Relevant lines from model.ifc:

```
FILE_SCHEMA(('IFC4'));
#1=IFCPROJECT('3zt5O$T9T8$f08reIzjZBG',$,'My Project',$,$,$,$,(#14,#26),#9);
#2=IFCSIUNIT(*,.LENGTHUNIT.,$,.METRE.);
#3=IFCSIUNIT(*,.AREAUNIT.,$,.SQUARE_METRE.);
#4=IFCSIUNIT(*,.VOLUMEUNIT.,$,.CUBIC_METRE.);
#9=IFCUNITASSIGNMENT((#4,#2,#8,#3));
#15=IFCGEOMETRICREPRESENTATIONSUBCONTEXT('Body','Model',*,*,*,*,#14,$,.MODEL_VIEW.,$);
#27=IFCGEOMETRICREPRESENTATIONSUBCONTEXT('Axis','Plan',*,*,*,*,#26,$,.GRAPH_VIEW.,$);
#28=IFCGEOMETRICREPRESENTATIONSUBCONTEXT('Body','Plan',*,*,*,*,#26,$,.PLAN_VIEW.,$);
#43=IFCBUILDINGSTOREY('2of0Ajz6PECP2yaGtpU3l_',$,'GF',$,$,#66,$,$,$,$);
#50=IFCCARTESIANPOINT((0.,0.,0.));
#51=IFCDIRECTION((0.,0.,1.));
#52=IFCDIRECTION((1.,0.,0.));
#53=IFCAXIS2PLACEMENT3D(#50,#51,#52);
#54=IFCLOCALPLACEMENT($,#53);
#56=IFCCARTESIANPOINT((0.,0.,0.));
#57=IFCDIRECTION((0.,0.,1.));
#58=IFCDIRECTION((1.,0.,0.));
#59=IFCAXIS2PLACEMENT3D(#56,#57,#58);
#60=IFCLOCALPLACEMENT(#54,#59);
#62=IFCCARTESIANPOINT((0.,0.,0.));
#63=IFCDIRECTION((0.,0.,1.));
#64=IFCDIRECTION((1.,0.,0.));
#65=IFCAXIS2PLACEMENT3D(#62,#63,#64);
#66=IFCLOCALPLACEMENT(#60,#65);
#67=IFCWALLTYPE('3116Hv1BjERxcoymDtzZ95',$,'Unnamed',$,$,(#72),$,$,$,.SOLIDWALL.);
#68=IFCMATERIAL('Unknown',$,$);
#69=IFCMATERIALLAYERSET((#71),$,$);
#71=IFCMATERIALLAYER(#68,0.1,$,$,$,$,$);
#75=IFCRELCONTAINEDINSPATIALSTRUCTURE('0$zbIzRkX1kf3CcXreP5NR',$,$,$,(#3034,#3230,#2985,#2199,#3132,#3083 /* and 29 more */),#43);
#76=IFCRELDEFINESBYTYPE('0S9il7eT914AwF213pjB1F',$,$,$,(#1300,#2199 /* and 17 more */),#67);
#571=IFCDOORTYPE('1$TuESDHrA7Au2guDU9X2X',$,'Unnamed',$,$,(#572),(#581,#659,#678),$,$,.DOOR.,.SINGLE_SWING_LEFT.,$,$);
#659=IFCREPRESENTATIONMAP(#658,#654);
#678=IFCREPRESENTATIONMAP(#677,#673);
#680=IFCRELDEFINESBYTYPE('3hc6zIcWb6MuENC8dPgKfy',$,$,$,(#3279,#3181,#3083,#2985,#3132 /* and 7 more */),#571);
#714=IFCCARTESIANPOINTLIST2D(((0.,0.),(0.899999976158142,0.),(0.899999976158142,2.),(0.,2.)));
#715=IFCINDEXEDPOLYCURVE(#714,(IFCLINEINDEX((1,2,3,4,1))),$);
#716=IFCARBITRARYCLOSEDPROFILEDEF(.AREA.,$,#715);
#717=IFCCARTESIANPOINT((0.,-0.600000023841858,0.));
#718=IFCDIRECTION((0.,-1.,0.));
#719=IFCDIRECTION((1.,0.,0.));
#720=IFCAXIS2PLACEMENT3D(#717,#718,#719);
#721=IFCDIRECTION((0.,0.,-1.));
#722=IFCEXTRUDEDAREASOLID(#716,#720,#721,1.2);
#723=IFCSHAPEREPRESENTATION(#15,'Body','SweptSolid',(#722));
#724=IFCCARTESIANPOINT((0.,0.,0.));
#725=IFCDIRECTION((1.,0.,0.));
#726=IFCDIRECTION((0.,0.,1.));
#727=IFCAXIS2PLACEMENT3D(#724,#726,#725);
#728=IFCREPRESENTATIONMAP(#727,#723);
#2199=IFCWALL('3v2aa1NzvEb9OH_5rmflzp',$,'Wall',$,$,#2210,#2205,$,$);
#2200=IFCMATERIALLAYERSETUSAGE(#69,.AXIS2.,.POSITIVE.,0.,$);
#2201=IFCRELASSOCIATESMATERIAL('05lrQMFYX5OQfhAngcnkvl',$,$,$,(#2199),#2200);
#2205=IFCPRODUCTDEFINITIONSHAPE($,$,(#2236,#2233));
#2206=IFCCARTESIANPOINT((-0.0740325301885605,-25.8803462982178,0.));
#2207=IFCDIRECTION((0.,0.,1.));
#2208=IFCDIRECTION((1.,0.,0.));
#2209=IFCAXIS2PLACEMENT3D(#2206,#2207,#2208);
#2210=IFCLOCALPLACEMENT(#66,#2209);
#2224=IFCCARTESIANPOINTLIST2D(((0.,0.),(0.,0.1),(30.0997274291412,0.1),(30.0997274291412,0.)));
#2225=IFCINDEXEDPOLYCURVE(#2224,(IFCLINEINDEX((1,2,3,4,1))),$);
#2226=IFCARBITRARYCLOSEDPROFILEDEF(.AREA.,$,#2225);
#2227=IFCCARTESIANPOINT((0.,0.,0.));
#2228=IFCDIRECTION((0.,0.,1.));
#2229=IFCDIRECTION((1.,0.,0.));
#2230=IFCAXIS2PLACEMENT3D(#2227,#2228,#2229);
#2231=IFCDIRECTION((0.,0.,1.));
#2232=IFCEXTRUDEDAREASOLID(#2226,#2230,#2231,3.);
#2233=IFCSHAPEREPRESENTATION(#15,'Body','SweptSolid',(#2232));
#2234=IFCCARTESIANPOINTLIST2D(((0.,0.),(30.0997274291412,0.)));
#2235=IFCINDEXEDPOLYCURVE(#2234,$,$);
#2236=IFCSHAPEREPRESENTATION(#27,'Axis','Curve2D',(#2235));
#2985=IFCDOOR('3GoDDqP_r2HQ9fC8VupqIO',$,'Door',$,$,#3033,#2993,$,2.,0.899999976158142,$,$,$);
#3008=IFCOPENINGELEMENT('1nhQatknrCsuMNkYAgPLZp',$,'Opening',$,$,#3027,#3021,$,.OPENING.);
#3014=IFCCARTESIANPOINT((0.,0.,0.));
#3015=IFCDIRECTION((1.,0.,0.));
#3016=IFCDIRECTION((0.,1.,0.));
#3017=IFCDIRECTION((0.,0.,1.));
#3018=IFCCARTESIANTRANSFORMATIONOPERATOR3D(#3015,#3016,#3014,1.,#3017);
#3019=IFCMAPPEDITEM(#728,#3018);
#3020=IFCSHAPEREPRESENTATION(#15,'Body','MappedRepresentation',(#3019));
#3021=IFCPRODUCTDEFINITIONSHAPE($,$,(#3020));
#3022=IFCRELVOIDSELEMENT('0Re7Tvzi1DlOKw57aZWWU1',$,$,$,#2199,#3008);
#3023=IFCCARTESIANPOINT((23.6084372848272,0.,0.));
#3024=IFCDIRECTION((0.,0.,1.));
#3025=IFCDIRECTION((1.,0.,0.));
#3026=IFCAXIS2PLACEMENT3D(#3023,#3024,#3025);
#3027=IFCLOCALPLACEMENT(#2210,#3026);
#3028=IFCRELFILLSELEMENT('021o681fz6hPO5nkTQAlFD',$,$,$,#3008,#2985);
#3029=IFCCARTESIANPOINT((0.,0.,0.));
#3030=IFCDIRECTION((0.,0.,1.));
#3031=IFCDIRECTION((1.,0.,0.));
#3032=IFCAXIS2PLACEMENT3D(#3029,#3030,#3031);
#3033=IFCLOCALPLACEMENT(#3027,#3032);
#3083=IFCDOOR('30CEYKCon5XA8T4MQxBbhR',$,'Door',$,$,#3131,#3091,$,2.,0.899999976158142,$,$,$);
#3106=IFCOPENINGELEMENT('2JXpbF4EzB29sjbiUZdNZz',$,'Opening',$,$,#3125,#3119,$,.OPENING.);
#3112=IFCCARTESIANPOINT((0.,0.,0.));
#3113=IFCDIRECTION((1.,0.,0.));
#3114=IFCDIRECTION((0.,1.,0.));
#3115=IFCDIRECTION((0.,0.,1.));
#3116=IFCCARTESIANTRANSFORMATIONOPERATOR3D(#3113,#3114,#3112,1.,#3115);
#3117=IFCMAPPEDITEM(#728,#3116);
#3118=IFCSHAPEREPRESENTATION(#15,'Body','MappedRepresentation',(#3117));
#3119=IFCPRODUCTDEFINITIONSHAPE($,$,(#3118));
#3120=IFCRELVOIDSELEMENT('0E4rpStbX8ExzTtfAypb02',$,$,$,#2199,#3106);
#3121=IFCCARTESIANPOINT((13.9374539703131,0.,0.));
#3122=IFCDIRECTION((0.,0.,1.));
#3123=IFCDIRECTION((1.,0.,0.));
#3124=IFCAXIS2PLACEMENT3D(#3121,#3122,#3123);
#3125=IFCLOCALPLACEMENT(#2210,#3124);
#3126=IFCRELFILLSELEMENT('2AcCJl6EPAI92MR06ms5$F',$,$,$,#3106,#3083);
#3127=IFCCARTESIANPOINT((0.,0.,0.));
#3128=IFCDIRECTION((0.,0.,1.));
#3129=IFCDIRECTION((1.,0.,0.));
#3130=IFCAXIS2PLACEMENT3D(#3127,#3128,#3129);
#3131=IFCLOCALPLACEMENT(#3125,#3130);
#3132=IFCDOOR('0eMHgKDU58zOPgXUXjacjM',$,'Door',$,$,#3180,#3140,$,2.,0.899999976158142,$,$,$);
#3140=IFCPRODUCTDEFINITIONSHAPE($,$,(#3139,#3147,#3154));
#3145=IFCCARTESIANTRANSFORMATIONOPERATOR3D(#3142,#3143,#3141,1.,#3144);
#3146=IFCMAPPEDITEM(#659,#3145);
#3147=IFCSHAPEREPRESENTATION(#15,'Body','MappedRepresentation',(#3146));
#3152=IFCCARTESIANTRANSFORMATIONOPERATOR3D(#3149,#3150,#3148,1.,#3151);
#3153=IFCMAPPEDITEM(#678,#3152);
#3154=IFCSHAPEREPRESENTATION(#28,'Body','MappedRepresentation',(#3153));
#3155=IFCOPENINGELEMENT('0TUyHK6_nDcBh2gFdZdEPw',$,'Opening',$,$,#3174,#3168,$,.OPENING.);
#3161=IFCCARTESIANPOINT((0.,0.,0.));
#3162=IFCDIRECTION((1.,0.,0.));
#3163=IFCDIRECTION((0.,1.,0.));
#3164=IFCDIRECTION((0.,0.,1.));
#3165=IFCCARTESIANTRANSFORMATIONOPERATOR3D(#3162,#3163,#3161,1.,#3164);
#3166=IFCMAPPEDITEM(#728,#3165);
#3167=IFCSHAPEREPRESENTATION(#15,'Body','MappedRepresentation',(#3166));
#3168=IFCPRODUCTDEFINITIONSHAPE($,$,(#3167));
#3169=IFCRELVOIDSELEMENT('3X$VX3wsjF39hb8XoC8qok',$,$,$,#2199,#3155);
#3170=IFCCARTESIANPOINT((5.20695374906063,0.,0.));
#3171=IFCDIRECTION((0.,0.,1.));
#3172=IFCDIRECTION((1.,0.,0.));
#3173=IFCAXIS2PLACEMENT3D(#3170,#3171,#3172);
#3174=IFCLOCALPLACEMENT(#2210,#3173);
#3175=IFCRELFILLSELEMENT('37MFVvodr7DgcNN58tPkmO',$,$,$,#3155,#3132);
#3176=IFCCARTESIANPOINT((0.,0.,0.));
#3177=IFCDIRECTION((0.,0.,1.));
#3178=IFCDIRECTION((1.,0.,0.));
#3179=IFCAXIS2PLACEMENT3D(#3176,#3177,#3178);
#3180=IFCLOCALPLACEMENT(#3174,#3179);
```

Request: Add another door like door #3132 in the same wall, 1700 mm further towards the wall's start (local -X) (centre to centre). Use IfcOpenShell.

```python
import ifcopenshell
import ifcopenshell.api.feature
import ifcopenshell.api.geometry
import ifcopenshell.api.root
import ifcopenshell.geom
import ifcopenshell.util.element
import ifcopenshell.util.placement
import ifcopenshell.util.shape

model = ifcopenshell.open("model.ifc")
settings = ifcopenshell.geom.settings()


def volume(element):
    """Net volume in cubic metres, openings subtracted."""
    shape = ifcopenshell.geom.create_shape(settings, element)
    return ifcopenshell.util.shape.get_volume(shape.geometry)


door = model.by_guid("0eMHgKDU58zOPgXUXjacjM")
opening = door.FillsVoids[0].RelatingOpeningElement
wall = opening.VoidsElements[0].RelatingBuildingElement
before = volume(wall)
shift = ifcopenshell.util.placement.get_local_placement(wall.ObjectPlacement)[:3, 0] * -1.7

# copy_class copies the void relationship, type, container and properties, but no geometry.
new_opening = ifcopenshell.api.root.copy_class(model, product=opening)
new_opening.Representation = ifcopenshell.util.element.copy_deep(
    model, opening.Representation, exclude=["IfcGeometricRepresentationContext", "IfcRepresentationMap"]
)
new_door = ifcopenshell.api.root.copy_class(model, product=door)
new_door.Representation = ifcopenshell.util.element.copy_deep(
    model, door.Representation, exclude=["IfcGeometricRepresentationContext", "IfcRepresentationMap"]
)
ifcopenshell.api.feature.add_filling(model, opening=new_opening, element=new_door)

for old, new in ((opening, new_opening), (door, new_door)):
    matrix = ifcopenshell.util.placement.get_local_placement(old.ObjectPlacement)
    matrix[:3, 3] += shift
    ifcopenshell.api.geometry.edit_object_placement(model, product=new, matrix=matrix, is_si=False)

after = volume(wall)

print(f"wall volume {before:.3f} -> {after:.3f} m3")

model.write("model_v2.ifc")
```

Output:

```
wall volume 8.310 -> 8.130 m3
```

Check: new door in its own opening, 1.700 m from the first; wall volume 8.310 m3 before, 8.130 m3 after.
